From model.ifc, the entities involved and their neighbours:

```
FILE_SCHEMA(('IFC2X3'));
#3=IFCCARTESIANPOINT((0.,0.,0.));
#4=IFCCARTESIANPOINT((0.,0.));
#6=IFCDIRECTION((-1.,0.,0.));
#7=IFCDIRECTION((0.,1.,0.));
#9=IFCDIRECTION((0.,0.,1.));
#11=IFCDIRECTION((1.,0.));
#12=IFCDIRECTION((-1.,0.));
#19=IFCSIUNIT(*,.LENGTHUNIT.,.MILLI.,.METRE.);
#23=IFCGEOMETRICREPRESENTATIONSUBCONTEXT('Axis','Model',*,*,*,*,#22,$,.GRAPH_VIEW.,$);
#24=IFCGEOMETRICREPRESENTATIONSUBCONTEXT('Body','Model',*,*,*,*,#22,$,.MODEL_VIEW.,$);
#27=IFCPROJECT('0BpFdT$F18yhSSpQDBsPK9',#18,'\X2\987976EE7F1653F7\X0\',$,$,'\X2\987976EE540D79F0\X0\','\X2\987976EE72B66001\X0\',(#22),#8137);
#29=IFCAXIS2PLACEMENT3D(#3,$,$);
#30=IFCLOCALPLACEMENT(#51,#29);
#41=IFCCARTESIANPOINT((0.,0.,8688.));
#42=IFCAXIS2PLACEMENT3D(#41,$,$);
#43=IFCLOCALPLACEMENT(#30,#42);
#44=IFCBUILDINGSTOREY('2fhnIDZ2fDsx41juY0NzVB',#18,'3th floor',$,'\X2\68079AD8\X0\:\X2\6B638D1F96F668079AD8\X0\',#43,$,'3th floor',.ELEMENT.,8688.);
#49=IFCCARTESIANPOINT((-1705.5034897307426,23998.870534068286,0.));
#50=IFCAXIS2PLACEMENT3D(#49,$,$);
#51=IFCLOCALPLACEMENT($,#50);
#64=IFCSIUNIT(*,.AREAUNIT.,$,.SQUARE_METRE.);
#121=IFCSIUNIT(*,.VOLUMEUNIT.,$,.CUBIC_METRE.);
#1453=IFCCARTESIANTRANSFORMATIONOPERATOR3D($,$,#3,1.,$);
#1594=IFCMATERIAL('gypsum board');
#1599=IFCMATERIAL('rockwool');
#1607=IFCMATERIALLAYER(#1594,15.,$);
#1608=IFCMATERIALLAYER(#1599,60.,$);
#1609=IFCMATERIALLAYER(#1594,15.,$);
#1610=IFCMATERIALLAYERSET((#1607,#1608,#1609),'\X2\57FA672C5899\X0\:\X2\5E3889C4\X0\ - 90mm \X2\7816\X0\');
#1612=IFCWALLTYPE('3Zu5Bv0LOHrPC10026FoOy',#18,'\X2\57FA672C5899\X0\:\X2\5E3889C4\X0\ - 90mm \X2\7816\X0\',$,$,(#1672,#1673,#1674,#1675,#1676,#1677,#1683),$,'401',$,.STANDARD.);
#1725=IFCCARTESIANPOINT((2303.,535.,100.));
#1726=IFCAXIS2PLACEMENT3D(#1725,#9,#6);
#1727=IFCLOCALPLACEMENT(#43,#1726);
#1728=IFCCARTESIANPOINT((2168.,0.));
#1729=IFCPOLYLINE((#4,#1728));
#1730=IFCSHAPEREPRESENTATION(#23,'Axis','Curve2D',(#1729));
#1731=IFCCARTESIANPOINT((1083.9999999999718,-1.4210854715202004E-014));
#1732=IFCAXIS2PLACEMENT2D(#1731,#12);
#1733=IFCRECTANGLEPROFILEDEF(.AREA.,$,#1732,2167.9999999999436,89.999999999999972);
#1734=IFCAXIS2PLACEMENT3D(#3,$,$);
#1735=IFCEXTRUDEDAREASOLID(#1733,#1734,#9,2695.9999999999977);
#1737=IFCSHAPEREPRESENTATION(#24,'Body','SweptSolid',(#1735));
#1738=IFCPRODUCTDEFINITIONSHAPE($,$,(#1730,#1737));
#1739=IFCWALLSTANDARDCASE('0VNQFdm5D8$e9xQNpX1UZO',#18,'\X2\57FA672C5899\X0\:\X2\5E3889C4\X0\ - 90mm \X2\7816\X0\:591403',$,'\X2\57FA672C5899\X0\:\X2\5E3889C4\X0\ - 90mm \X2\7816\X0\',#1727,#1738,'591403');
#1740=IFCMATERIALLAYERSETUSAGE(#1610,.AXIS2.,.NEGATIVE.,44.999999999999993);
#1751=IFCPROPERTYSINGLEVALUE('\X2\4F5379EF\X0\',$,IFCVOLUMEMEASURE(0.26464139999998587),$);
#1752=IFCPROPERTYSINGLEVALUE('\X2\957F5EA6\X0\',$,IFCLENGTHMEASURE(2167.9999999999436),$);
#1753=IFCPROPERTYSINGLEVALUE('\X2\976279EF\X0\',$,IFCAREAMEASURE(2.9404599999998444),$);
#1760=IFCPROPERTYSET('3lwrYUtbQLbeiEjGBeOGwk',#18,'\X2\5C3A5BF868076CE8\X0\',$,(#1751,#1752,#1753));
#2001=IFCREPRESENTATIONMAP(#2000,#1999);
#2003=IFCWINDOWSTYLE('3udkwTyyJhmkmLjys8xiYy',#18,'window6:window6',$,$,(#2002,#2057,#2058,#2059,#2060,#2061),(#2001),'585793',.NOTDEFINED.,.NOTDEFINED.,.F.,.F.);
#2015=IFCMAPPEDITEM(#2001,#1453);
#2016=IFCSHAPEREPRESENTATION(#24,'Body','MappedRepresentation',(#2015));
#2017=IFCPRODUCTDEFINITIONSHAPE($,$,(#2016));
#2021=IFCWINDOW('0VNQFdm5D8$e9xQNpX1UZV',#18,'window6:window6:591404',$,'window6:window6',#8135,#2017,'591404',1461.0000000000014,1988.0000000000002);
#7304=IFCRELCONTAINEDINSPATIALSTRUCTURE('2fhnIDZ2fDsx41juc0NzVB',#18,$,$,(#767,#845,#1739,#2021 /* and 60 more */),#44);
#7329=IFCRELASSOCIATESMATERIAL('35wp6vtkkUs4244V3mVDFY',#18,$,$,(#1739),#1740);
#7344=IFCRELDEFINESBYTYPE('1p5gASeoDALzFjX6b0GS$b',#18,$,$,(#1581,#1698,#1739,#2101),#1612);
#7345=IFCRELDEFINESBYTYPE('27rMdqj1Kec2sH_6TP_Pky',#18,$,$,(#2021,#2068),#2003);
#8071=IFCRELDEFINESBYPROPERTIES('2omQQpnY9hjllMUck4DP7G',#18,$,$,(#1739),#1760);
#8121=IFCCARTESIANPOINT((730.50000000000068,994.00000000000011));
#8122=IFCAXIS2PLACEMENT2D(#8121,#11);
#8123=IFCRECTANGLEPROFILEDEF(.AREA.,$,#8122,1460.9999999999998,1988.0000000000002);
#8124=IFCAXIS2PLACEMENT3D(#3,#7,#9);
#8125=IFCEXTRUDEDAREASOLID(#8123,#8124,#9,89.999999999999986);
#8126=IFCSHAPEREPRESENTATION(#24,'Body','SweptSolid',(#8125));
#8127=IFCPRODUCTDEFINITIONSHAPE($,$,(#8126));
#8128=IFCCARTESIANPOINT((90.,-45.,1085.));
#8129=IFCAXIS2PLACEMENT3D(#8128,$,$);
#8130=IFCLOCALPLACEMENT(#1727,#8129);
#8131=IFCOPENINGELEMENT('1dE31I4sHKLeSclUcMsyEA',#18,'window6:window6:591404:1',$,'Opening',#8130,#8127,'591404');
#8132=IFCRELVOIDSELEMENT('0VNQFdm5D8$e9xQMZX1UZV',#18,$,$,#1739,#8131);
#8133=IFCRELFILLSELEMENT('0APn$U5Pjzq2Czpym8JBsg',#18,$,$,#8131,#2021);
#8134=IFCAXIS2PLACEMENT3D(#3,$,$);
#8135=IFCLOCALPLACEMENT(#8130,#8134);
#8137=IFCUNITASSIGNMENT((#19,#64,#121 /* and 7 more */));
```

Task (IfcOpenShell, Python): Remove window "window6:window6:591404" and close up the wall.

```python
import ifcopenshell
import ifcopenshell.api.feature
import ifcopenshell.api.pset
import ifcopenshell.api.root
import ifcopenshell.geom
import ifcopenshell.util.element
import ifcopenshell.util.shape
import ifcopenshell.util.unit

model = ifcopenshell.open("model.ifc")
area_scale = ifcopenshell.util.unit.calculate_unit_scale(model, "AREAUNIT")
volume_scale = ifcopenshell.util.unit.calculate_unit_scale(model, "VOLUMEUNIT")
settings = ifcopenshell.geom.settings()


def volume(element):
    """Net volume in cubic metres, openings subtracted."""
    shape = ifcopenshell.geom.create_shape(settings, element)
    return ifcopenshell.util.shape.get_volume(shape.geometry)


window = model.by_guid("0VNQFdm5D8$e9xQNpX1UZV")
opening = window.FillsVoids[0].RelatingOpeningElement
wall = opening.VoidsElements[0].RelatingBuildingElement
before = volume(wall)

ifcopenshell.api.root.remove_product(model, product=window)
ifcopenshell.api.feature.remove_feature(model, feature=opening)

after = volume(wall)
thickness = 0.09  # wall thickness in metres

# Update the wall's stored quantities.
pset = model.by_id(ifcopenshell.util.element.get_pset(wall, "尺寸标注", should_inherit=False)["id"])
ifcopenshell.api.pset.edit_pset(model, pset=pset, properties={
    "体积": model.create_entity("IfcVolumeMeasure", after / volume_scale),
    "面积": model.create_entity("IfcAreaMeasure", after / thickness / area_scale),
})

print(f"wall volume {before:.3f} -> {after:.3f} m3")

model.write("model_v2.ifc")
```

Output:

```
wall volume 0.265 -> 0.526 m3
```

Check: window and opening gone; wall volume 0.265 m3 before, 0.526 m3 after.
